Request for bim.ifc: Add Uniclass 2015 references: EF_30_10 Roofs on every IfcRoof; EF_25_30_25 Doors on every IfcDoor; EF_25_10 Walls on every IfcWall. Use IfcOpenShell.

First a look at what the model holds.

```python
import ifcopenshell

model = ifcopenshell.open("bim.ifc")
print(model.schema)
print("classifications:", [c.Name for c in model.by_type("IfcClassification")])
for ifc_class in ("IfcDoor", "IfcRoof", "IfcStair", "IfcWall", "IfcWindow"):
    print(ifc_class, len(model.by_type(ifc_class)))
```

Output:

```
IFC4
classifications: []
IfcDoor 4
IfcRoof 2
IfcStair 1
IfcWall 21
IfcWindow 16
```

```python
import ifcopenshell
import ifcopenshell.api.classification

model = ifcopenshell.open("bim.ifc")

system = ifcopenshell.api.classification.add_classification(model, classification="Uniclass 2015")

codes = {
    "IfcRoof": ("EF_30_10", "Roofs"),
    "IfcDoor": ("EF_25_30_25", "Doors"),
    "IfcWall": ("EF_25_10", "Walls"),
}
for ifc_class, (code, name) in codes.items():
    products = model.by_type(ifc_class)
    ifcopenshell.api.classification.add_reference(
        model, products=products, classification=system, identification=code, name=name
    )
    print(code, len(products))

model.write("bim_edited.ifc")
```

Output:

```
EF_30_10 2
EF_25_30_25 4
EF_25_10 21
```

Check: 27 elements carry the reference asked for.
